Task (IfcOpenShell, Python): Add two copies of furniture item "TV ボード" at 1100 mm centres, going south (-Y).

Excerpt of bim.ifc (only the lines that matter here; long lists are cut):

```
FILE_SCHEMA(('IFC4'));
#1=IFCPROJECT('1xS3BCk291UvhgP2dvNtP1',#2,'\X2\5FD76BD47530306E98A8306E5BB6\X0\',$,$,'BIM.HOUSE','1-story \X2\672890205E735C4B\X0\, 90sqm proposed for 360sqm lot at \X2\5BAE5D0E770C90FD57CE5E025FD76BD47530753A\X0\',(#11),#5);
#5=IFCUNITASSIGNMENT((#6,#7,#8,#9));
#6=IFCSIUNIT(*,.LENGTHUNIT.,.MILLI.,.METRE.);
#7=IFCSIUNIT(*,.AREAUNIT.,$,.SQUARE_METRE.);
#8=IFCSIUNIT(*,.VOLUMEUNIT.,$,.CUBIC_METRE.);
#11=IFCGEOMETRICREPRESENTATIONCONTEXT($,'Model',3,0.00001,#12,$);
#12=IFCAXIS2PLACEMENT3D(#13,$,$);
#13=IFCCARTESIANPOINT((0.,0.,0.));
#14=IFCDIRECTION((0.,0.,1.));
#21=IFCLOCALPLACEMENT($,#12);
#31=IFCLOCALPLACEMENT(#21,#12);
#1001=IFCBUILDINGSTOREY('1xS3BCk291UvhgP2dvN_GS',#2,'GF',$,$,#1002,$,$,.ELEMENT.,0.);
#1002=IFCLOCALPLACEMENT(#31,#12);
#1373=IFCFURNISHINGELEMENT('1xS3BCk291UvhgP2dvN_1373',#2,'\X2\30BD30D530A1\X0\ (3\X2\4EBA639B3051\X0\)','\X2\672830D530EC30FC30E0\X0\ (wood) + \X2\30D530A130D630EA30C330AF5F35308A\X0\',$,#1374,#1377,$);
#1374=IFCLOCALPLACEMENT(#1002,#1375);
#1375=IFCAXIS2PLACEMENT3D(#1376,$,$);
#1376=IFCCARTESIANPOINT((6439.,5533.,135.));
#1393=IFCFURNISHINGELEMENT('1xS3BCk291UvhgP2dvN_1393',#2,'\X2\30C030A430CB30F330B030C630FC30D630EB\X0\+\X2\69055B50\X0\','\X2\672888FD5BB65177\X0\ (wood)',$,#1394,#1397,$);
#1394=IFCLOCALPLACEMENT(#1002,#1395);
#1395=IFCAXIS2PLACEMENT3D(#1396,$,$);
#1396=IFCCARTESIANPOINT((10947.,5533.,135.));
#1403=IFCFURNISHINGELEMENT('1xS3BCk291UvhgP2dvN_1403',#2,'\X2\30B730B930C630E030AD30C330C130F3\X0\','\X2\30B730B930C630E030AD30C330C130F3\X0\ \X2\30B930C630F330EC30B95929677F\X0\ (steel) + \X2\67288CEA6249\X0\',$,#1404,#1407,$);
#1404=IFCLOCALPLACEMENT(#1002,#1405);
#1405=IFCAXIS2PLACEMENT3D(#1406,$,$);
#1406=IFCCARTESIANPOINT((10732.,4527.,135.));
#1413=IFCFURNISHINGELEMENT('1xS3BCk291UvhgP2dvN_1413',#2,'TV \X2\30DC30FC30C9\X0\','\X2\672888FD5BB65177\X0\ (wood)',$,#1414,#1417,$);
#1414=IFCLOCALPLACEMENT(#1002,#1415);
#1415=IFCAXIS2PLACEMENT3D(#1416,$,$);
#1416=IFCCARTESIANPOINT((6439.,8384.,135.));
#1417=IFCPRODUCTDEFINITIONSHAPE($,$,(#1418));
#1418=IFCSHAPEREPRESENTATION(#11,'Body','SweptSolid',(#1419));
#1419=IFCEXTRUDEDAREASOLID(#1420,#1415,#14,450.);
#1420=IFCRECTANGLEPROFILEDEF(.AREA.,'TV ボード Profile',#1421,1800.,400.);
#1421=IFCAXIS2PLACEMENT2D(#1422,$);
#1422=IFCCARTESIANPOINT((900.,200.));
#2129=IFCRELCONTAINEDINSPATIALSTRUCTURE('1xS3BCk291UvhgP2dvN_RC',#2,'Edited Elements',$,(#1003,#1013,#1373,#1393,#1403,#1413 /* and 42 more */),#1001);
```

```python
import numpy as np
import ifcopenshell
import ifcopenshell.api.geometry
import ifcopenshell.api.root
import ifcopenshell.util.element
import ifcopenshell.util.placement
import ifcopenshell.util.unit

model = ifcopenshell.open("bim.ifc")
unit_scale = ifcopenshell.util.unit.calculate_unit_scale(model)


def reuse_history(source, copy):
    """copy_class also copies each property set's owner history, people and application; keep the originals."""
    for rel in copy.IsDefinedBy:
        if rel.is_a("IfcRelDefinesByProperties") and (history := rel.RelatingPropertyDefinition.OwnerHistory):
            rel.RelatingPropertyDefinition.OwnerHistory = source.OwnerHistory
            ifcopenshell.util.element.remove_deep2(model, history)


source = model.by_guid("1xS3BCk291UvhgP2dvN_1413")
base = ifcopenshell.util.placement.get_local_placement(source.ObjectPlacement)
step = np.array([0.0, -1.0, 0.0]) * 1.1 / unit_scale

for i in range(1, 3):
    copy = ifcopenshell.api.root.copy_class(model, product=source)
    copy.Representation = ifcopenshell.util.element.copy_deep(
        model, source.Representation, exclude=["IfcGeometricRepresentationContext", "IfcRepresentationMap"]
    )
    reuse_history(source, copy)
    matrix = base.copy()
    matrix[:3, 3] += i * step
    print("added at", matrix[:3, 3].round(3) + 0.0)
    ifcopenshell.api.geometry.edit_object_placement(model, product=copy, matrix=matrix, is_si=False)

model.write("bim_edited.ifc")
```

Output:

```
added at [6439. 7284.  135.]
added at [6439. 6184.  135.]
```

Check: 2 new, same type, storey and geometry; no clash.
